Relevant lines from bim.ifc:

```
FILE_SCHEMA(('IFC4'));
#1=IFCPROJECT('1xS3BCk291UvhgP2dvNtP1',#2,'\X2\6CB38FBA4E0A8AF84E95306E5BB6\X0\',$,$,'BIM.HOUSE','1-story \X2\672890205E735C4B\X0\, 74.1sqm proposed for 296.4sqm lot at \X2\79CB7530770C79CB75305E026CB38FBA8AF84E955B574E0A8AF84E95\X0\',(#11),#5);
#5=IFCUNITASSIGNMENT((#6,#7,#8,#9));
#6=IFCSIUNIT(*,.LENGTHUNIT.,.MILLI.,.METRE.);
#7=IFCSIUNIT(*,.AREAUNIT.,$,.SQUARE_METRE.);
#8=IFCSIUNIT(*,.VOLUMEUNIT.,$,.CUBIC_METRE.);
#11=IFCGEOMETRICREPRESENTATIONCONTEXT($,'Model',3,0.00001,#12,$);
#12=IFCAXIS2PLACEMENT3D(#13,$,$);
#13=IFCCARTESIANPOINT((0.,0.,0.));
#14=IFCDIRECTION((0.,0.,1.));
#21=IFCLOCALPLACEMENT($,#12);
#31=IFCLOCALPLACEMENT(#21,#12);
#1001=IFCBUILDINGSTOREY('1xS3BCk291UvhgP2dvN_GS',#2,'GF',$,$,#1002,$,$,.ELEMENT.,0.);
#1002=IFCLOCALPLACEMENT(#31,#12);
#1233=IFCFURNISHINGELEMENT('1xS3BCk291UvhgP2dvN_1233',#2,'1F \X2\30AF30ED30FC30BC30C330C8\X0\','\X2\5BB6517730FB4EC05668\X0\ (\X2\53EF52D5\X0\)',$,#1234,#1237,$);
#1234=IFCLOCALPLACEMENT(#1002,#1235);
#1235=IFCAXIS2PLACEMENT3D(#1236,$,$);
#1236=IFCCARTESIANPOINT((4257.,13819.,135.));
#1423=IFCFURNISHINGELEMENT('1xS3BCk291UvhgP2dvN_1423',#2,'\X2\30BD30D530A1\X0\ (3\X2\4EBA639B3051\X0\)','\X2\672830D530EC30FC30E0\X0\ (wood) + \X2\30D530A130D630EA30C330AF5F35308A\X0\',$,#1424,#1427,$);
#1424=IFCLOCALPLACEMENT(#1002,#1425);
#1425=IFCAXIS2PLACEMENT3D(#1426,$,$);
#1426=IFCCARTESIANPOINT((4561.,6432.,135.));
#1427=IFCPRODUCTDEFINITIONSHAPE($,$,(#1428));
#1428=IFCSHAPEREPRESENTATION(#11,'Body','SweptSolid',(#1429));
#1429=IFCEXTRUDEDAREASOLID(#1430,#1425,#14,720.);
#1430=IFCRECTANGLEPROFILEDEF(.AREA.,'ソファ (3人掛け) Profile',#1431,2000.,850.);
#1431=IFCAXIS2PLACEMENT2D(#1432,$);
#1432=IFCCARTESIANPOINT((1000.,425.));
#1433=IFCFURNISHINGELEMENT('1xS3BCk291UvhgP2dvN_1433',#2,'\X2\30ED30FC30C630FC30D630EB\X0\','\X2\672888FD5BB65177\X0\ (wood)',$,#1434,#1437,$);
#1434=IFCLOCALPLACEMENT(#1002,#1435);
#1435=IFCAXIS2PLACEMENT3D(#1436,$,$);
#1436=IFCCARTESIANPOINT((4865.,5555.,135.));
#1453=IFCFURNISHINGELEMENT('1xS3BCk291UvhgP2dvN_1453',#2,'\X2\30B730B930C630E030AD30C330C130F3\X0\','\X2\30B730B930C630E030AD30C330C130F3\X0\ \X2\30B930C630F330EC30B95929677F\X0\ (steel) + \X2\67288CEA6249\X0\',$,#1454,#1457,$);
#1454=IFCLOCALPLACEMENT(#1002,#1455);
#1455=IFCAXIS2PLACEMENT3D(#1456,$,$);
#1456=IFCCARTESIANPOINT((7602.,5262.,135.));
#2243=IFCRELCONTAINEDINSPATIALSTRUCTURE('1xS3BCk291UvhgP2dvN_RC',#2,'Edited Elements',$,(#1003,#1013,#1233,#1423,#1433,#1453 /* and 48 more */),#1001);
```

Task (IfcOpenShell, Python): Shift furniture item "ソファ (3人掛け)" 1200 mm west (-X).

```python
import ifcopenshell
import ifcopenshell.api.geometry
import ifcopenshell.util.placement

model = ifcopenshell.open("bim.ifc")

item = model.by_guid("1xS3BCk291UvhgP2dvN_1423")
matrix = ifcopenshell.util.placement.get_local_placement(item.ObjectPlacement)
matrix[0, 3] -= 1200.0
ifcopenshell.api.geometry.edit_object_placement(model, product=item, matrix=matrix, is_si=False)

print(ifcopenshell.util.placement.get_local_placement(item.ObjectPlacement).round(3) + 0.0)

model.write("bim_v2.ifc")
```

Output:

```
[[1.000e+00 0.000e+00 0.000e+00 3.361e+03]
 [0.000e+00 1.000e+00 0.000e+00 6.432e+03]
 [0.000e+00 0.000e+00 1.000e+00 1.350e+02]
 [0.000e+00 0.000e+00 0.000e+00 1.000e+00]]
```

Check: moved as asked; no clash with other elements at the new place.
